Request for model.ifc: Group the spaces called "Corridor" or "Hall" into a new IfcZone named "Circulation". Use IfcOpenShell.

First a look at what the model holds.

```python
import ifcopenshell

model = ifcopenshell.open("model.ifc")
print(model.schema)
seen = {}
for space in model.by_type("IfcSpace"):
    seen[space.LongName] = seen.get(space.LongName, 0) + 1
for name, count in sorted(seen.items(), key=str):
    print(count, "x", name)
print("zones:", [z.Name for z in model.by_type("IfcZone")][:20])
```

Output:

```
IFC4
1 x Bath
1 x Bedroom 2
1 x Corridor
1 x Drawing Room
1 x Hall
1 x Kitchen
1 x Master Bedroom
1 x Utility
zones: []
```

```python
import ifcopenshell
import ifcopenshell.api.group
import ifcopenshell.api.root

model = ifcopenshell.open("model.ifc")

names = {"Corridor", "Hall"}
spaces = [s for s in model.by_type("IfcSpace") if s.LongName in names]

zone = ifcopenshell.api.root.create_entity(model, ifc_class="IfcZone", name="Circulation")
ifcopenshell.api.group.assign_group(model, products=spaces, group=zone)
print(len(spaces), "spaces in", zone.Name)

model.write("model_edited.ifc")
```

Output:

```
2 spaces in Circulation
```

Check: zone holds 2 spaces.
